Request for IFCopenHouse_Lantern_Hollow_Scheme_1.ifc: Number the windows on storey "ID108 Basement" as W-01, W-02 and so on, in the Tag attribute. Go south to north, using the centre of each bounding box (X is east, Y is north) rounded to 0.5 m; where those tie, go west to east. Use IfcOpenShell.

First a look at what the model holds.

```python
import ifcopenshell
import ifcopenshell.util.element
import ifcopenshell.util.placement

model = ifcopenshell.open("IFCopenHouse_Lantern_Hollow_Scheme_1.ifc")
print(model.schema)
storey = next(s for s in model.by_type("IfcBuildingStorey") if s.Name == "ID108 Basement")
windows = [e for e in ifcopenshell.util.element.get_decomposition(storey) if e.is_a("IfcWindow")]
for e in sorted(windows, key=lambda e: e.id()):
    origin = ifcopenshell.util.placement.get_local_placement(e.ObjectPlacement)[:3, 3]
    print(e.id(), e.Tag, e.Name, origin.round(2) + 0.0, sep=" | ")
```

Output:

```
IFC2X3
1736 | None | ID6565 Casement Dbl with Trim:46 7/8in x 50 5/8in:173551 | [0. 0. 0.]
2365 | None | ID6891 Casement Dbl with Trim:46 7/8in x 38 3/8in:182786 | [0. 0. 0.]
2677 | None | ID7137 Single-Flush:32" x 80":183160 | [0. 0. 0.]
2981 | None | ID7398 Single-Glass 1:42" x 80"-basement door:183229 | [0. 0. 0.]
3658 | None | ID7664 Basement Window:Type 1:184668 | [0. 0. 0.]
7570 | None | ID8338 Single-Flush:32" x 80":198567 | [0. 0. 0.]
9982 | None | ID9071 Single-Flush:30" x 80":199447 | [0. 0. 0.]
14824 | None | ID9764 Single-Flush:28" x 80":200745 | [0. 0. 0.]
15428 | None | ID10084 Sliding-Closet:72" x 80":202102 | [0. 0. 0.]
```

```python
import ifcopenshell
import ifcopenshell.geom
import ifcopenshell.util.element
import ifcopenshell.util.shape

model = ifcopenshell.open("IFCopenHouse_Lantern_Hollow_Scheme_1.ifc")
settings = ifcopenshell.geom.settings()
settings.set("use-world-coords", True)


def centre(element):
    shape = ifcopenshell.geom.create_shape(settings, element)
    return ifcopenshell.util.shape.get_bbox_centroid(shape.geometry)


storey = next(s for s in model.by_type("IfcBuildingStorey") if s.Name == "ID108 Basement")
windows = [e for e in ifcopenshell.util.element.get_decomposition(storey) if e.is_a("IfcWindow")]

# Insertion points can sit at a corner or the storey origin, so sort by the geometry (in metres).
centres = {e: centre(e) for e in windows}
windows.sort(key=lambda e: (round(centres[e][1] / 0.5), centres[e][0]))

for i, e in enumerate(windows, start=1):
    number = f"W-{i:02d}"
    e.Tag = number
    print(e.id(), number)

model.write("IFCopenHouse_Lantern_Hollow_Scheme_1_rev.ifc")
```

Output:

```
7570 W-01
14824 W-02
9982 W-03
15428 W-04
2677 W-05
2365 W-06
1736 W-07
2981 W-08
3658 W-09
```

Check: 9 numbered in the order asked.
